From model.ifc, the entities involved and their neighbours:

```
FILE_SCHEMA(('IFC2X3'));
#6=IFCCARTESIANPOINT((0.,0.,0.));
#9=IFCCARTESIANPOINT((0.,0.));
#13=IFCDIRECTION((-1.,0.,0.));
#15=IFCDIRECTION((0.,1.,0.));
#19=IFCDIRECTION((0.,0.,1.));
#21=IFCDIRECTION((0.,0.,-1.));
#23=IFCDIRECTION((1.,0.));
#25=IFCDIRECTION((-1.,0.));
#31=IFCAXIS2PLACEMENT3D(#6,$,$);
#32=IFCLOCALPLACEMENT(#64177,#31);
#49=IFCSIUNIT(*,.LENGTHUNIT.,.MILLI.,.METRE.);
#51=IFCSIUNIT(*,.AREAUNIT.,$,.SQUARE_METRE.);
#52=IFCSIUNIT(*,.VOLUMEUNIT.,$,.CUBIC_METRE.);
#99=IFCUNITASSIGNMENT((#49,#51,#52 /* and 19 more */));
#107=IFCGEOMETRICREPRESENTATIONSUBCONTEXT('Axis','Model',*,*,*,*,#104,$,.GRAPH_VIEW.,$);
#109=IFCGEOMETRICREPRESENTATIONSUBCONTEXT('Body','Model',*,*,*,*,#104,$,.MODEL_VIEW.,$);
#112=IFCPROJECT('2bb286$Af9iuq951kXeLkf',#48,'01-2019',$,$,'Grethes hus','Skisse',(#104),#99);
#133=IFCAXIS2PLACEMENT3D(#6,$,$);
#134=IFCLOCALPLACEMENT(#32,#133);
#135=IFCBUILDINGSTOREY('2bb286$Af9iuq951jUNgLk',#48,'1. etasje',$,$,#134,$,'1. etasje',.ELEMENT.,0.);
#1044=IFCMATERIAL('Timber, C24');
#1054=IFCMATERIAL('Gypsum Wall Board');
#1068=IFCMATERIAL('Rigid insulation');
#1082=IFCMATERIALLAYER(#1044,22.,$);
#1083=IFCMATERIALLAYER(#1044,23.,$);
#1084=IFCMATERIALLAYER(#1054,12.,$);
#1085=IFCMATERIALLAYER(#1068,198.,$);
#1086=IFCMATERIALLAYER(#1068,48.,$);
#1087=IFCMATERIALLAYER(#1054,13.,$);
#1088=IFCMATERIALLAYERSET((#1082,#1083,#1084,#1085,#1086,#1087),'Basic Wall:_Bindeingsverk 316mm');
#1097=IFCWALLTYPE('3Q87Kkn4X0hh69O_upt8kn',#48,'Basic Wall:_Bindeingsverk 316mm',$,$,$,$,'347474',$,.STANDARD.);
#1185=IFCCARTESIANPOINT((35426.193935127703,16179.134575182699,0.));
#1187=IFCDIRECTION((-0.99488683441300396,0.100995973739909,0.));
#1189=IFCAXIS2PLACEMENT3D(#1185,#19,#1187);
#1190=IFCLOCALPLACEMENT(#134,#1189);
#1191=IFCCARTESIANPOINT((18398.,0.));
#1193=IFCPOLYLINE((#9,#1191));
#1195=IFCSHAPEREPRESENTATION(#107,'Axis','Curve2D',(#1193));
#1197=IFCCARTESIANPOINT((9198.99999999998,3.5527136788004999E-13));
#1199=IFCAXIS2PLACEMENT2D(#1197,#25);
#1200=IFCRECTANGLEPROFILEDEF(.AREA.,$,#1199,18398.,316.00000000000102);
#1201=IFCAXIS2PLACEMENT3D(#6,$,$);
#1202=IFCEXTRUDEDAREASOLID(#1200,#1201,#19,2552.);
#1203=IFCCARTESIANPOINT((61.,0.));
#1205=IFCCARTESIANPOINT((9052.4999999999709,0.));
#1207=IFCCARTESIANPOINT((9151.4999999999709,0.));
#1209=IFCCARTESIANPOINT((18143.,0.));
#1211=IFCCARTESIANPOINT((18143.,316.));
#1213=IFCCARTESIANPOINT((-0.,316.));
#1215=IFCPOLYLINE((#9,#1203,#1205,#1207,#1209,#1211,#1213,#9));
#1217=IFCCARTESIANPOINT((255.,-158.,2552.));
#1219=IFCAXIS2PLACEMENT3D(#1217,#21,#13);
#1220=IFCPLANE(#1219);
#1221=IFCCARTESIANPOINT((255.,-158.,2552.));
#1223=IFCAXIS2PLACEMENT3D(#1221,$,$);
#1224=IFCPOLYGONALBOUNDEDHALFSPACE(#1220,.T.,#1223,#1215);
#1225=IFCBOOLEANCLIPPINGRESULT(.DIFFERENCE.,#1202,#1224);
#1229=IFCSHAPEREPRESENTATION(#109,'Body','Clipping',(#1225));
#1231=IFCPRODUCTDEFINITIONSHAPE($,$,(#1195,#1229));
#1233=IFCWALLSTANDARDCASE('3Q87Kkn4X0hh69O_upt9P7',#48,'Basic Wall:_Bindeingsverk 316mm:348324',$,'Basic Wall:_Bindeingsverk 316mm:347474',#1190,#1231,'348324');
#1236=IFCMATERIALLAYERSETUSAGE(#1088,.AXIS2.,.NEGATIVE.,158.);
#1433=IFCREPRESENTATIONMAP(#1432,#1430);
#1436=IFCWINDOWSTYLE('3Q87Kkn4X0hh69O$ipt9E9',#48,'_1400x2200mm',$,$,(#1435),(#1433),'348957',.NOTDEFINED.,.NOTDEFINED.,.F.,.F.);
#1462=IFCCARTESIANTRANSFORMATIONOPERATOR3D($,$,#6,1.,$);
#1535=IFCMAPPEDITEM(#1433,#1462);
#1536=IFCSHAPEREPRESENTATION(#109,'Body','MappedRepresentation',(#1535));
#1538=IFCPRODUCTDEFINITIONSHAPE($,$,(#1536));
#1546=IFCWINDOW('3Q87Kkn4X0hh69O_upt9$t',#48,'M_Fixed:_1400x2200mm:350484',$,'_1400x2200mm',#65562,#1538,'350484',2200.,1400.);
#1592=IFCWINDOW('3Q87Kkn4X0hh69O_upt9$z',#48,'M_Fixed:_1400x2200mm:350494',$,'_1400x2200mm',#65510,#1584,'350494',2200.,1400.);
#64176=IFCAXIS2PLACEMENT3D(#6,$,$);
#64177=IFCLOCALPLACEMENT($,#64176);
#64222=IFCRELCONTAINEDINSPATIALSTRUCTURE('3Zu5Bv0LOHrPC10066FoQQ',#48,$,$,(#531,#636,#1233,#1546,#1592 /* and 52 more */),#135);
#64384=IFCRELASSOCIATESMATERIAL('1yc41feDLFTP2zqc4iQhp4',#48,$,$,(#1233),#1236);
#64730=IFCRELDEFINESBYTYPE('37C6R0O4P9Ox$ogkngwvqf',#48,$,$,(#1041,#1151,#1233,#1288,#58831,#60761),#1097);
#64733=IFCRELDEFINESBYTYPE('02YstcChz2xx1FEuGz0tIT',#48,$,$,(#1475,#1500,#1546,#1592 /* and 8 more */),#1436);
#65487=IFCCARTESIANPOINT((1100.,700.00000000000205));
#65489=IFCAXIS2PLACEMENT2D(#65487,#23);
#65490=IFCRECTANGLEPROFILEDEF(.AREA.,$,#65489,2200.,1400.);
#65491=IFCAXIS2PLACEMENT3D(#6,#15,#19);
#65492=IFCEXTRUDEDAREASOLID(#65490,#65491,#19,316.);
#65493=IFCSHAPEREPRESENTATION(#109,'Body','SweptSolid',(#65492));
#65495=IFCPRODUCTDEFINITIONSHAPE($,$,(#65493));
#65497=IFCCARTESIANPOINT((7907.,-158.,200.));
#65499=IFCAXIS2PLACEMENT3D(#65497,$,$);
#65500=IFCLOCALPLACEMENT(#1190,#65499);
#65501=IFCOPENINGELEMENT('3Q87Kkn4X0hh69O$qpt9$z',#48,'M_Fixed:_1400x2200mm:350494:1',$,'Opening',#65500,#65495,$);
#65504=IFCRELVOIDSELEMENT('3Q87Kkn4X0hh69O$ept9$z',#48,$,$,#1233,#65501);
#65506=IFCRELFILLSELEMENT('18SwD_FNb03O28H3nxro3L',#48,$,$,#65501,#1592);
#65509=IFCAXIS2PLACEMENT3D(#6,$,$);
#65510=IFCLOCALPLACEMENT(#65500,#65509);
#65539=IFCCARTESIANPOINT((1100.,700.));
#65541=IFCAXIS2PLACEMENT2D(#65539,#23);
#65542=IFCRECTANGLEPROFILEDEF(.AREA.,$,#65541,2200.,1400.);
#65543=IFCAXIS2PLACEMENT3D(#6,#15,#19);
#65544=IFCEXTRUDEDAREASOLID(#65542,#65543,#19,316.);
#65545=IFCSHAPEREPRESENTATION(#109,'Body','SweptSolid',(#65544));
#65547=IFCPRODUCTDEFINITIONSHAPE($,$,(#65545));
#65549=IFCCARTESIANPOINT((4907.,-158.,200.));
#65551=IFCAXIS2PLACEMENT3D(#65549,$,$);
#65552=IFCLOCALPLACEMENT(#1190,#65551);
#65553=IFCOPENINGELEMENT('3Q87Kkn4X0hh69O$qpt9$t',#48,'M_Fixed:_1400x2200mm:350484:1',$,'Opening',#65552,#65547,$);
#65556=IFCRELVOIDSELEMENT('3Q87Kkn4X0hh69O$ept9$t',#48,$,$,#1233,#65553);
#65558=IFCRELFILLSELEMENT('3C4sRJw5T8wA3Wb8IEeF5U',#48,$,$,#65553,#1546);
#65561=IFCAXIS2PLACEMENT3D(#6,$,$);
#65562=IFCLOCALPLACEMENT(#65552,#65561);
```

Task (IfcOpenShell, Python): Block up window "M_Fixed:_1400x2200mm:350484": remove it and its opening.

```python
import ifcopenshell
import ifcopenshell.api.feature
import ifcopenshell.api.root
import ifcopenshell.geom
import ifcopenshell.util.shape

model = ifcopenshell.open("model.ifc")
settings = ifcopenshell.geom.settings()


def volume(element):
    """Net volume in cubic metres, openings subtracted."""
    shape = ifcopenshell.geom.create_shape(settings, element)
    return ifcopenshell.util.shape.get_volume(shape.geometry)


window = model.by_guid("3Q87Kkn4X0hh69O_upt9$t")
opening = window.FillsVoids[0].RelatingOpeningElement
wall = opening.VoidsElements[0].RelatingBuildingElement
before = volume(wall)

ifcopenshell.api.root.remove_product(model, product=window)
ifcopenshell.api.feature.remove_feature(model, feature=opening)

after = volume(wall)

print(f"wall volume {before:.3f} -> {after:.3f} m3")

model.write("model-out.ifc")
```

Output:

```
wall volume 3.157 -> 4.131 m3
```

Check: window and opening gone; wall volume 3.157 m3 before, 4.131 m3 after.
